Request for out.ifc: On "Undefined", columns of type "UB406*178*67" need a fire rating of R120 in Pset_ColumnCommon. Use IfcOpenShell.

First a look at what the model holds.

```python
import ifcopenshell
import ifcopenshell.util.element

model = ifcopenshell.open("out.ifc")
print(model.schema)
storey = next(s for s in model.by_type("IfcBuildingStorey") if s.Name == "Undefined")
columns = [e for e in ifcopenshell.util.element.get_decomposition(storey) if e.is_a("IfcColumn")]
seen = {}
for e in columns:
    element_type = ifcopenshell.util.element.get_type(e)
    key = (element_type.Name if element_type != e and element_type else None, ifcopenshell.util.element.get_pset(e, "Pset_ColumnCommon", "FireRating"))
    seen[key] = seen.get(key, 0) + 1
for (name, value), count in sorted(seen.items(), key=str):
    print(count, "x", name, "|", value)
```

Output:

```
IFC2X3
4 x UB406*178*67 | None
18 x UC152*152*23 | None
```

```python
import ifcopenshell
import ifcopenshell.api.pset
import ifcopenshell.util.element

model = ifcopenshell.open("out.ifc")

storey = next(s for s in model.by_type("IfcBuildingStorey") if s.Name == "Undefined")
columns = [e for e in ifcopenshell.util.element.get_decomposition(storey) if e.is_a("IfcColumn")]

count = 0
for e in columns:
    element_type = ifcopenshell.util.element.get_type(e)
    if element_type in (None, e) or element_type.Name != "UB406*178*67":
        continue
    found = ifcopenshell.util.element.get_pset(e, "Pset_ColumnCommon", should_inherit=False)
    if found:
        pset = model.by_id(found["id"])
        if len(ifcopenshell.util.element.get_elements_by_pset(pset)) > 1:
            pset = ifcopenshell.api.pset.unshare_pset(model, products=[e], pset=pset)[0]
    else:
        pset = ifcopenshell.api.pset.add_pset(model, product=e, name="Pset_ColumnCommon")
    ifcopenshell.api.pset.edit_pset(model, pset=pset, properties={"FireRating": "R120"})
    count += 1

print(count, "columns updated")

model.write("out_updated.ifc")
```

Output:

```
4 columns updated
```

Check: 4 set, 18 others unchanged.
